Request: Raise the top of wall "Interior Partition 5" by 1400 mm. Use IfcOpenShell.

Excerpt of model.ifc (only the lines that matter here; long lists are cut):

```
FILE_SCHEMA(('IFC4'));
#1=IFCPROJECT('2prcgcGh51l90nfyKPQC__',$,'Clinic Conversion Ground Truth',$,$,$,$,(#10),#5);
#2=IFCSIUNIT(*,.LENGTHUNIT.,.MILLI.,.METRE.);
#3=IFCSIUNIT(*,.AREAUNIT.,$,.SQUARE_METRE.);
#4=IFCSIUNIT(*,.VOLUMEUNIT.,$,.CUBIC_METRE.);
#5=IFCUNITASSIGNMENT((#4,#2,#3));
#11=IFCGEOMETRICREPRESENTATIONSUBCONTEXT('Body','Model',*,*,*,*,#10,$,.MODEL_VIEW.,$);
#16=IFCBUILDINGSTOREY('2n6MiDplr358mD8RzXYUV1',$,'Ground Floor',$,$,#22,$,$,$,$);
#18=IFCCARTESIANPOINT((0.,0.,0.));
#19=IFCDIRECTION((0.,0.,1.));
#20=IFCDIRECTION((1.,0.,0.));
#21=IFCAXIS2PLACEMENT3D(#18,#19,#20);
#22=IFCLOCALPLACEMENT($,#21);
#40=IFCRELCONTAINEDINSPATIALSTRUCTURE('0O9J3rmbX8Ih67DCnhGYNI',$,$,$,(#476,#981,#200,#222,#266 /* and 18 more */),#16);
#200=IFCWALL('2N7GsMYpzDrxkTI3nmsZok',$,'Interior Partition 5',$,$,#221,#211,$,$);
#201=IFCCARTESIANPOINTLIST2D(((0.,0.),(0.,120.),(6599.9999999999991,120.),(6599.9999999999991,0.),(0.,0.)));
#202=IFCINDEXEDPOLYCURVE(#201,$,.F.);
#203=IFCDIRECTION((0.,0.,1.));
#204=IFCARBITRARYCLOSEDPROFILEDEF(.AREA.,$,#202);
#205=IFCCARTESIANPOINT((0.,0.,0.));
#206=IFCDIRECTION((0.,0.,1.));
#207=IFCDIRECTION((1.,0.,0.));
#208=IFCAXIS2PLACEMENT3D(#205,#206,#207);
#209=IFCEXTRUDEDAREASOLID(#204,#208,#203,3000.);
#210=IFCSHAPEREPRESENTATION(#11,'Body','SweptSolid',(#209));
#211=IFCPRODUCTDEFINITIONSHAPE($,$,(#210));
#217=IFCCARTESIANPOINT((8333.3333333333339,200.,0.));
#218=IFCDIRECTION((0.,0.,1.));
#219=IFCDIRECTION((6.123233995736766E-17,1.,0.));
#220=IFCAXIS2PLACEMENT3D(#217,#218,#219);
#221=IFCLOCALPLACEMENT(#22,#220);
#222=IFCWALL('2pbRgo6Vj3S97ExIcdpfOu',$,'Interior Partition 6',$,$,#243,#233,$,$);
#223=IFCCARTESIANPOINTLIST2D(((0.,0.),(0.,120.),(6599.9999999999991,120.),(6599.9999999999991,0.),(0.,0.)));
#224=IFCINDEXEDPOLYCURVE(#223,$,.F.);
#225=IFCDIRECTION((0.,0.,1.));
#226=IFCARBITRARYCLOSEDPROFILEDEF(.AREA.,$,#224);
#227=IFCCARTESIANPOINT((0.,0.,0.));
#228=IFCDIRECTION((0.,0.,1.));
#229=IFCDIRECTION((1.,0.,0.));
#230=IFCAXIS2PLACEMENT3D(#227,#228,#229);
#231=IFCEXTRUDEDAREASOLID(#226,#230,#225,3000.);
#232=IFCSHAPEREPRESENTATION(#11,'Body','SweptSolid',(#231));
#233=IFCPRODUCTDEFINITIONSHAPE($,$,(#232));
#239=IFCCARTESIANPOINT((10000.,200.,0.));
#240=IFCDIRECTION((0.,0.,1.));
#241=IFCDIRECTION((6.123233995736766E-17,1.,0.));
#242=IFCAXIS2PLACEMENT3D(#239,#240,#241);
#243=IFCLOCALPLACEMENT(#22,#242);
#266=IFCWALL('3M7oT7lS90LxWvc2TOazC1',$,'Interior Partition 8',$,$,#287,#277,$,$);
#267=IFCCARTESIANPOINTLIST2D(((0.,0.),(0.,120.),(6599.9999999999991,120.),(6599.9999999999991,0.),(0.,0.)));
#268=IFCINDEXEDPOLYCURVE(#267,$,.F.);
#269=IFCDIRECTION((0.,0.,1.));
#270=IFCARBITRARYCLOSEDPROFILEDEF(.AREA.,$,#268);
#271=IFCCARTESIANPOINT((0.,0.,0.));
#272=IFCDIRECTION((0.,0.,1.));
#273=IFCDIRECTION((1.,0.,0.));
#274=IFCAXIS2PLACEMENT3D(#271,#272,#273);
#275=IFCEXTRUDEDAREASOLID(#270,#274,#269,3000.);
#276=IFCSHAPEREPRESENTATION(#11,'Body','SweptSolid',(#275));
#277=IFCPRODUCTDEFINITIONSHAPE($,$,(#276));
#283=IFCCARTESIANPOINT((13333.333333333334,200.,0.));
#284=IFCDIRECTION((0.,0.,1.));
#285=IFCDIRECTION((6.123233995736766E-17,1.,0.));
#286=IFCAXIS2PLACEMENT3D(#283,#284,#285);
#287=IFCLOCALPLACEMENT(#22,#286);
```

```python
import ifcopenshell
import ifcopenshell.geom
import ifcopenshell.util.representation
import ifcopenshell.util.shape
import ifcopenshell.util.unit

model = ifcopenshell.open("model.ifc")
unit_scale = ifcopenshell.util.unit.calculate_unit_scale(model)
settings = ifcopenshell.geom.settings()


def volume(element):
    """Net volume in cubic metres, openings subtracted."""
    shape = ifcopenshell.geom.create_shape(settings, element)
    return ifcopenshell.util.shape.get_volume(shape.geometry)


wall = model.by_guid("2N7GsMYpzDrxkTI3nmsZok")
before = volume(wall)

body = ifcopenshell.util.representation.get_representation(wall, "Model", "Body")
solid = body.Items[0]
old_height = solid.Depth
solid.Depth += 1.4 / unit_scale
after = volume(wall)

print(f"height {old_height:g} -> {solid.Depth:g}, volume {before:.3f} -> {after:.3f} m3")

model.write("model-out.ifc")
```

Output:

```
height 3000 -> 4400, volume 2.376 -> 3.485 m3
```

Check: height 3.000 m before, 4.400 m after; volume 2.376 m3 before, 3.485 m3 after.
